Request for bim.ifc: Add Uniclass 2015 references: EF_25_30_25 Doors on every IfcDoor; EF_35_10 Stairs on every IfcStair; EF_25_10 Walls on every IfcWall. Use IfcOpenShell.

First a look at what the model holds.

```python
import ifcopenshell

model = ifcopenshell.open("bim.ifc")
print(model.schema)
print("classifications:", [c.Name for c in model.by_type("IfcClassification")])
for ifc_class in ("IfcDoor", "IfcRoof", "IfcStair", "IfcWall", "IfcWindow"):
    print(ifc_class, len(model.by_type(ifc_class)))
```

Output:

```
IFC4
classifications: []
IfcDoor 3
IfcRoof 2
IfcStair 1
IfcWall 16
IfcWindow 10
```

```python
import ifcopenshell
import ifcopenshell.api.classification

model = ifcopenshell.open("bim.ifc")

system = ifcopenshell.api.classification.add_classification(model, classification="Uniclass 2015")

codes = {
    "IfcDoor": ("EF_25_30_25", "Doors"),
    "IfcStair": ("EF_35_10", "Stairs"),
    "IfcWall": ("EF_25_10", "Walls"),
}
for ifc_class, (code, name) in codes.items():
    products = model.by_type(ifc_class)
    ifcopenshell.api.classification.add_reference(
        model, products=products, classification=system, identification=code, name=name
    )
    print(code, len(products))

model.write("bim-out.ifc")
```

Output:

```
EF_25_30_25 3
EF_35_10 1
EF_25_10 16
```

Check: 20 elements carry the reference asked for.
